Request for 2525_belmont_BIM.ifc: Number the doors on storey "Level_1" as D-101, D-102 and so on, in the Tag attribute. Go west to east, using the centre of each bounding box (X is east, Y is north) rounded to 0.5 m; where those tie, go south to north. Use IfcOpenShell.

First a look at what the model holds.

```python
import ifcopenshell
import ifcopenshell.util.element
import ifcopenshell.util.placement

model = ifcopenshell.open("2525_belmont_BIM.ifc")
print(model.schema)
storey = next(s for s in model.by_type("IfcBuildingStorey") if s.Name == "Level_1")
doors = [e for e in ifcopenshell.util.element.get_decomposition(storey) if e.is_a("IfcDoor")]
for e in sorted(doors, key=lambda e: e.id()):
    origin = ifcopenshell.util.placement.get_local_placement(e.ObjectPlacement)[:3, 3]
    print(e.id(), e.Tag, e.Name, origin.round(2) + 0.0, sep=" | ")
```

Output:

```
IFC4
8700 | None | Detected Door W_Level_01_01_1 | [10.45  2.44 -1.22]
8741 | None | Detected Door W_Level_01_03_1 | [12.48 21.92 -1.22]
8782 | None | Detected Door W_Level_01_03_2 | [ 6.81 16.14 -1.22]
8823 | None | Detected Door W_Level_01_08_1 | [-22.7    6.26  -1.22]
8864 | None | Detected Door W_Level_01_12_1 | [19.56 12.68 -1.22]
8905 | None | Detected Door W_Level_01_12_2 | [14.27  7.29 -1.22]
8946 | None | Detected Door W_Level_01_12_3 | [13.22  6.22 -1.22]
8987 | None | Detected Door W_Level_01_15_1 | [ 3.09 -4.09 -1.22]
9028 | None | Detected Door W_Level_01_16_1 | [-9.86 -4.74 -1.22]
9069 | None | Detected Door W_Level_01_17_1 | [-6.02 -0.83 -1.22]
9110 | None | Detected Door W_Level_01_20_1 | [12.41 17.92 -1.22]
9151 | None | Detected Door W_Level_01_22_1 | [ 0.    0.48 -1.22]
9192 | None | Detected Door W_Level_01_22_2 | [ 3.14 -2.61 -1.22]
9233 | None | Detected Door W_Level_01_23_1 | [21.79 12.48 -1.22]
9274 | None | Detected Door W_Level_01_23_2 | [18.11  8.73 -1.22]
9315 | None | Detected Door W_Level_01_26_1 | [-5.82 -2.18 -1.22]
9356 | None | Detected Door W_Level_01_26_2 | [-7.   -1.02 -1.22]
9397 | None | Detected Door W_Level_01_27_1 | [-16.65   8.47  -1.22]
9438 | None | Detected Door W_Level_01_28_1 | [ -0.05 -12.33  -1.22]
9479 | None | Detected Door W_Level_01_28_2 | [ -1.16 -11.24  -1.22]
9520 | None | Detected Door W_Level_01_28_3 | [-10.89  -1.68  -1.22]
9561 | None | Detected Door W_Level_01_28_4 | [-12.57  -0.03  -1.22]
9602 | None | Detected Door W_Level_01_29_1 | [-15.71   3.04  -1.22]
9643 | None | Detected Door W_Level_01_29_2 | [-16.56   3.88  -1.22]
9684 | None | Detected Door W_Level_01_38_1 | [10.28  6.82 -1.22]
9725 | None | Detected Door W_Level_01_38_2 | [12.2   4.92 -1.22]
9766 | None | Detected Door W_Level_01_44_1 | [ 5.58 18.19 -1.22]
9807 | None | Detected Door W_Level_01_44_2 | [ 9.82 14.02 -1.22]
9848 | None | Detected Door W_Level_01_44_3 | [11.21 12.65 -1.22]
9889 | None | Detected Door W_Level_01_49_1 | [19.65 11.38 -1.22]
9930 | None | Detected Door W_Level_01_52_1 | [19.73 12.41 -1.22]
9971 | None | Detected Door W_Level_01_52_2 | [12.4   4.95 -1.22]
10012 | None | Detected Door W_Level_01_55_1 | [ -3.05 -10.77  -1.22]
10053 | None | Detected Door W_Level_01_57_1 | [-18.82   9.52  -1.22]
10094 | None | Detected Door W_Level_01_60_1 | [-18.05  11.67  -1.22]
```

```python
import ifcopenshell
import ifcopenshell.geom
import ifcopenshell.util.element
import ifcopenshell.util.shape

model = ifcopenshell.open("2525_belmont_BIM.ifc")
settings = ifcopenshell.geom.settings()
settings.set("use-world-coords", True)


def centre(element):
    shape = ifcopenshell.geom.create_shape(settings, element)
    return ifcopenshell.util.shape.get_bbox_centroid(shape.geometry)


storey = next(s for s in model.by_type("IfcBuildingStorey") if s.Name == "Level_1")
doors = [e for e in ifcopenshell.util.element.get_decomposition(storey) if e.is_a("IfcDoor")]

# Insertion points can sit at a corner or the storey origin, so sort by the geometry (in metres).
centres = {e: centre(e) for e in doors}
doors.sort(key=lambda e: (round(centres[e][0] / 0.5), centres[e][1]))

for i, e in enumerate(doors, start=1):
    number = f"D-1{i:02d}"
    e.Tag = number
    print(e.id(), number)

model.write("2525_belmont_BIM_updated.ifc")
```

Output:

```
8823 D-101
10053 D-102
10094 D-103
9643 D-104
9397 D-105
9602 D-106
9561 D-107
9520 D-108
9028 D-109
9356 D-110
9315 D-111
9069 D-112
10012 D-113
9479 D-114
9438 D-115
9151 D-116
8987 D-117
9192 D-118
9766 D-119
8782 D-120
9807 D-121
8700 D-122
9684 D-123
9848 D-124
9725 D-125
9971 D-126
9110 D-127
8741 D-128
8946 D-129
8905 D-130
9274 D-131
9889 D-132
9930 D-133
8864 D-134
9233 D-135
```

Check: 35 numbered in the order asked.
